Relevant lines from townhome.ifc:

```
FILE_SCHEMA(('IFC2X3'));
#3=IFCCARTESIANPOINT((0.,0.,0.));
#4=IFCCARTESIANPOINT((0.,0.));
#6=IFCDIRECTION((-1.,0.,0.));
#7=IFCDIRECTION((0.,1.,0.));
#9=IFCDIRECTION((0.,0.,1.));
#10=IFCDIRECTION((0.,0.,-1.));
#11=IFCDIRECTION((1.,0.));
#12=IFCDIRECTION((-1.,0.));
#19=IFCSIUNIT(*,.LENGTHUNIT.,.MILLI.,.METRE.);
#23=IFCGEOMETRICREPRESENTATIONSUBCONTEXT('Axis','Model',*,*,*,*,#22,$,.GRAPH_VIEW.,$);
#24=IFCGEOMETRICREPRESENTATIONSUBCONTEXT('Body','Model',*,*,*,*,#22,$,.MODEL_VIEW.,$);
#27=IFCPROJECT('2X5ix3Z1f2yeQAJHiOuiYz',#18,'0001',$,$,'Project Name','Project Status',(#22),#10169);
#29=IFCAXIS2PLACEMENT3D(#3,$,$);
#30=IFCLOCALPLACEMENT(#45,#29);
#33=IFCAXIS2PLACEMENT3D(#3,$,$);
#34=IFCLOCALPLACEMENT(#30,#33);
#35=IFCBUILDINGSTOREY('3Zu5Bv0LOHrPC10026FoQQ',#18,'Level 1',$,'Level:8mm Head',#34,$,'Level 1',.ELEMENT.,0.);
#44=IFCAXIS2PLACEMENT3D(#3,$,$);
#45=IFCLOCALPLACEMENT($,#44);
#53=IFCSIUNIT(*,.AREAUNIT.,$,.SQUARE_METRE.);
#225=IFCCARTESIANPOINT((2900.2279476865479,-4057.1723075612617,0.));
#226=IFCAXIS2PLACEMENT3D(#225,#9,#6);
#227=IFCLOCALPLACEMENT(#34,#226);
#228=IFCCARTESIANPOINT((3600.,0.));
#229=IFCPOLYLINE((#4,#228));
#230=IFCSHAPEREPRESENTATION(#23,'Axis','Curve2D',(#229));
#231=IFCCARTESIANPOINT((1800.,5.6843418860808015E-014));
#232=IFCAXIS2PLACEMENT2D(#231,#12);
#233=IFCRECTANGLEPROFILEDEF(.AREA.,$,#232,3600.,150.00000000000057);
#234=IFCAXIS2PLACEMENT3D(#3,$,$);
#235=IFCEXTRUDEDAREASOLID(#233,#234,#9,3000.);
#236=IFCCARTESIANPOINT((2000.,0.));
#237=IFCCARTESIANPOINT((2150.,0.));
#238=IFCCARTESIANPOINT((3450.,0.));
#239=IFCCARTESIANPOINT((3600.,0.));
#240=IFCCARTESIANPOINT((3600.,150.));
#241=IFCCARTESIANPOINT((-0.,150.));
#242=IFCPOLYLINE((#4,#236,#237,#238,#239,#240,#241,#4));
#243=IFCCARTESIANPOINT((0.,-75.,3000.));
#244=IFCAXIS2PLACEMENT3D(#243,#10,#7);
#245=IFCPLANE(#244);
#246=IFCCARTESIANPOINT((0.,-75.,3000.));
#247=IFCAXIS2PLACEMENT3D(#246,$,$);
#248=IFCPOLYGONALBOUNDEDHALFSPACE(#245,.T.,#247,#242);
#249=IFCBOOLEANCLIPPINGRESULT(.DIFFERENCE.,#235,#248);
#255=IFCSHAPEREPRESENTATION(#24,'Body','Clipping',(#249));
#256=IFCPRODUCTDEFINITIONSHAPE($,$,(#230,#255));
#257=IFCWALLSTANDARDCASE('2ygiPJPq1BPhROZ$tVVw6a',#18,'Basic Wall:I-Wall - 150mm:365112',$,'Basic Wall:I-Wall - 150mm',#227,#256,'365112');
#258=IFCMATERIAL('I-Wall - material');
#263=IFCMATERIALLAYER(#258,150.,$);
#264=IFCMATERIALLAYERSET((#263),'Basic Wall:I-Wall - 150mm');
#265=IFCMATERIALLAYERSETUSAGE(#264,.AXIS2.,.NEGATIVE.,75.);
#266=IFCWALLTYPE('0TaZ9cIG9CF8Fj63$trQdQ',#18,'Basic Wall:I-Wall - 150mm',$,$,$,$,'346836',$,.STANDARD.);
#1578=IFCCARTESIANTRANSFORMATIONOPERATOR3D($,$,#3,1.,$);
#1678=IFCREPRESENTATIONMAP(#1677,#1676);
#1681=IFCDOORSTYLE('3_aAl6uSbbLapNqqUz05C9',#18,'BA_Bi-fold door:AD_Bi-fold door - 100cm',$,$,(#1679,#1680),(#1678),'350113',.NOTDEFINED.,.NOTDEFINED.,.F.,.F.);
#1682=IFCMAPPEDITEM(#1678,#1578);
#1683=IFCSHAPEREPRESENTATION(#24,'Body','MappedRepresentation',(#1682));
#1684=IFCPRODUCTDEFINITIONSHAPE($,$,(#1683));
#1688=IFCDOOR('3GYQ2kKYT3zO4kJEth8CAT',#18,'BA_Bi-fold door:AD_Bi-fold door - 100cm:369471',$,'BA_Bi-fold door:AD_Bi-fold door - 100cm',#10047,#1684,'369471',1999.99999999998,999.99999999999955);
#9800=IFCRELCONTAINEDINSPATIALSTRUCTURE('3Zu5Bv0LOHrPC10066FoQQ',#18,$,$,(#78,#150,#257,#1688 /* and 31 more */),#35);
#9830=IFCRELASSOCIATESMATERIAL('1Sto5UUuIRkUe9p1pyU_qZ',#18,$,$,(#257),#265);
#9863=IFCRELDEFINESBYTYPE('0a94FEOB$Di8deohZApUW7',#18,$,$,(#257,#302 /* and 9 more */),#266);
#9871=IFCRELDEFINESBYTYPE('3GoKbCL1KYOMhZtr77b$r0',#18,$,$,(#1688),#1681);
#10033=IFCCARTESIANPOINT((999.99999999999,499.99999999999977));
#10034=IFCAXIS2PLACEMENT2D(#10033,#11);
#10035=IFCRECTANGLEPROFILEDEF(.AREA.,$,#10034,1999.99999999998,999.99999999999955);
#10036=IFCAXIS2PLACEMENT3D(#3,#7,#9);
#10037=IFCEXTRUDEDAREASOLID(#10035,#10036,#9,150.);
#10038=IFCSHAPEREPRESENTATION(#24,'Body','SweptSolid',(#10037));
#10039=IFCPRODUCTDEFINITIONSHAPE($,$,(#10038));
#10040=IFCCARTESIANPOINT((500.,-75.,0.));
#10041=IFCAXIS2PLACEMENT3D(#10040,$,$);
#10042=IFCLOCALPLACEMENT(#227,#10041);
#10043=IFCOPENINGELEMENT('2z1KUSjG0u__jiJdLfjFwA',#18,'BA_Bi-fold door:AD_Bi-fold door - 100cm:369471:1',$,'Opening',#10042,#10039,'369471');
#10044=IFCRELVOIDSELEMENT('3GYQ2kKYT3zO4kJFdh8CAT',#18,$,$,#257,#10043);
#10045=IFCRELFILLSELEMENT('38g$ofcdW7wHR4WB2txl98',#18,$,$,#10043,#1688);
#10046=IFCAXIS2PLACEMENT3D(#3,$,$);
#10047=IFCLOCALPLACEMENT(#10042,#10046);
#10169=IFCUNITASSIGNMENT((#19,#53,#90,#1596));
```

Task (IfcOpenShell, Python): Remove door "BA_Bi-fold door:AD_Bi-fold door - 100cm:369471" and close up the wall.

```python
import ifcopenshell
import ifcopenshell.api.feature
import ifcopenshell.api.root
import ifcopenshell.geom
import ifcopenshell.util.shape

model = ifcopenshell.open("townhome.ifc")
settings = ifcopenshell.geom.settings()


def volume(element):
    """Net volume in cubic metres, openings subtracted."""
    shape = ifcopenshell.geom.create_shape(settings, element)
    return ifcopenshell.util.shape.get_volume(shape.geometry)


door = model.by_guid("3GYQ2kKYT3zO4kJEth8CAT")
opening = door.FillsVoids[0].RelatingOpeningElement
wall = opening.VoidsElements[0].RelatingBuildingElement
before = volume(wall)

ifcopenshell.api.root.remove_product(model, product=door)
ifcopenshell.api.feature.remove_feature(model, feature=opening)

after = volume(wall)

print(f"wall volume {before:.3f} -> {after:.3f} m3")

model.write("townhome_updated.ifc")
```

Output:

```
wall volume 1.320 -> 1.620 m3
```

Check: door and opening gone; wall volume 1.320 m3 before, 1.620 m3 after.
